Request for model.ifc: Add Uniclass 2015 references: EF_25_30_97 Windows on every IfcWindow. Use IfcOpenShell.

First a look at what the model holds.

```python
import ifcopenshell

model = ifcopenshell.open("model.ifc")
print(model.schema)
print("classifications:", [c.Name for c in model.by_type("IfcClassification")])
for ifc_class in ("IfcDoor", "IfcRoof", "IfcStair", "IfcWall", "IfcWindow"):
    print(ifc_class, len(model.by_type(ifc_class)))
```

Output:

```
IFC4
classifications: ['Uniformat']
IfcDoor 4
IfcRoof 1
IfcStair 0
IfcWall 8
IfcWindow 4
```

```python
import ifcopenshell
import ifcopenshell.api.classification

model = ifcopenshell.open("model.ifc")

system = ifcopenshell.api.classification.add_classification(model, classification="Uniclass 2015")

codes = {
    "IfcWindow": ("EF_25_30_97", "Windows"),
}
for ifc_class, (code, name) in codes.items():
    products = model.by_type(ifc_class)
    ifcopenshell.api.classification.add_reference(
        model, products=products, classification=system, identification=code, name=name
    )
    print(code, len(products))

model.write("model_v2.ifc")
```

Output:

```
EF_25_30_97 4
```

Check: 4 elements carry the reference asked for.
